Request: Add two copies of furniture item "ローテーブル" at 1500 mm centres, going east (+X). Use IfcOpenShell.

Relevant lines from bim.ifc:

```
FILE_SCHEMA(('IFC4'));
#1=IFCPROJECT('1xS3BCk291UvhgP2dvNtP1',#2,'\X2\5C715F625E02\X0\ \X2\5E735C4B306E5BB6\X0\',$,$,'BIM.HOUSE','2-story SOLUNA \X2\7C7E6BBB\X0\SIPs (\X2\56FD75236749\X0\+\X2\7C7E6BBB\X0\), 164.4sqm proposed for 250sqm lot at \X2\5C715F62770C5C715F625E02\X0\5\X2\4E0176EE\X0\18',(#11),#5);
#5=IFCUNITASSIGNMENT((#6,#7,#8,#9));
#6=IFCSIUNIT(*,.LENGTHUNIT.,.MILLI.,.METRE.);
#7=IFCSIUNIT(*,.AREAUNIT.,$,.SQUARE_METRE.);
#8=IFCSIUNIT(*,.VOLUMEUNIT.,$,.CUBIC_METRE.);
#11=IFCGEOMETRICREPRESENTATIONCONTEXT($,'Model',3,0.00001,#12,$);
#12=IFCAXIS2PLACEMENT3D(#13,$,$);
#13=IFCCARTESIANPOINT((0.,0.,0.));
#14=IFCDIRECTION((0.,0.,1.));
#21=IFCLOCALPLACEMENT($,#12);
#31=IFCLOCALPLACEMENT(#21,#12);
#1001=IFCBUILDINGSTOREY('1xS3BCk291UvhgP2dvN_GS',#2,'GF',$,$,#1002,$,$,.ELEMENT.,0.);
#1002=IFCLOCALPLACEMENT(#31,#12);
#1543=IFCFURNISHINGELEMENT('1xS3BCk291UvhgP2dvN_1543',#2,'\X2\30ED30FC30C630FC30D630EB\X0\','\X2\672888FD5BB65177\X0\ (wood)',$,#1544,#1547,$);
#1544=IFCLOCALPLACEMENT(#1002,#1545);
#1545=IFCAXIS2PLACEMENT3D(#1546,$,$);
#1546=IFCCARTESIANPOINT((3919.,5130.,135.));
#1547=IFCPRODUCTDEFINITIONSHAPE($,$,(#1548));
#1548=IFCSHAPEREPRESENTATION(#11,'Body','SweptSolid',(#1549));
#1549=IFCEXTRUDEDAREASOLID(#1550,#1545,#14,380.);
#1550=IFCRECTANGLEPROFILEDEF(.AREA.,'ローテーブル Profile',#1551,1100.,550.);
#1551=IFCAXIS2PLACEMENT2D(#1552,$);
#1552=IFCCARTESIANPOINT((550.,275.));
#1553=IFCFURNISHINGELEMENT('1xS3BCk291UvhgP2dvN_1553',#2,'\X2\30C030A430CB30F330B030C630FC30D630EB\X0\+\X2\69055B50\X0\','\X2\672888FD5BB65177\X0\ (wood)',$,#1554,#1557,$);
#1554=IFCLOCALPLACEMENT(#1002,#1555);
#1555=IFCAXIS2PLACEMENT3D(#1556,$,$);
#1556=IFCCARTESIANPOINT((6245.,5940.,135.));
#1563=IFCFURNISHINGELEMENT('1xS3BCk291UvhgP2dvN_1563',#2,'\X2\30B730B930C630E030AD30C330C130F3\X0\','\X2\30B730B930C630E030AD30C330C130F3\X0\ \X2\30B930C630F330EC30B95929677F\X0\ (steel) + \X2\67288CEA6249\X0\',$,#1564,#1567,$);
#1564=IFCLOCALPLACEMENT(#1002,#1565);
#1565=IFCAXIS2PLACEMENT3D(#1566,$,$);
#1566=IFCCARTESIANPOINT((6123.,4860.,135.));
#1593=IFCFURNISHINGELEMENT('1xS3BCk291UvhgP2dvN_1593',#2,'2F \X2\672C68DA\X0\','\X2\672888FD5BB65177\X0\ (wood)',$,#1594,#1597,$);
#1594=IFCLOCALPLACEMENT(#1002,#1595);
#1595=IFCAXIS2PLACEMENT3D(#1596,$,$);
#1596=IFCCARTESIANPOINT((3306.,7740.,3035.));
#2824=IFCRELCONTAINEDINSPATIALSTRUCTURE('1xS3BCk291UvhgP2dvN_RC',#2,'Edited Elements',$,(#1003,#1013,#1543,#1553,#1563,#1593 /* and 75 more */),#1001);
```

```python
import numpy as np
import ifcopenshell
import ifcopenshell.api.geometry
import ifcopenshell.api.root
import ifcopenshell.util.element
import ifcopenshell.util.placement
import ifcopenshell.util.unit

model = ifcopenshell.open("bim.ifc")
unit_scale = ifcopenshell.util.unit.calculate_unit_scale(model)


def reuse_history(source, copy):
    """copy_class also copies each property set's owner history, people and application; keep the originals."""
    for rel in copy.IsDefinedBy:
        if rel.is_a("IfcRelDefinesByProperties") and (history := rel.RelatingPropertyDefinition.OwnerHistory):
            rel.RelatingPropertyDefinition.OwnerHistory = source.OwnerHistory
            ifcopenshell.util.element.remove_deep2(model, history)


source = model.by_guid("1xS3BCk291UvhgP2dvN_1543")
base = ifcopenshell.util.placement.get_local_placement(source.ObjectPlacement)
step = np.array([1.0, 0.0, 0.0]) * 1.5 / unit_scale

for i in range(1, 3):
    copy = ifcopenshell.api.root.copy_class(model, product=source)
    copy.Representation = ifcopenshell.util.element.copy_deep(
        model, source.Representation, exclude=["IfcGeometricRepresentationContext", "IfcRepresentationMap"]
    )
    reuse_history(source, copy)
    matrix = base.copy()
    matrix[:3, 3] += i * step
    print("added at", matrix[:3, 3].round(3) + 0.0)
    ifcopenshell.api.geometry.edit_object_placement(model, product=copy, matrix=matrix, is_si=False)

model.write("bim_rev.ifc")
```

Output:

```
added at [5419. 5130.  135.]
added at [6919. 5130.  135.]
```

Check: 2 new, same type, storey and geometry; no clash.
